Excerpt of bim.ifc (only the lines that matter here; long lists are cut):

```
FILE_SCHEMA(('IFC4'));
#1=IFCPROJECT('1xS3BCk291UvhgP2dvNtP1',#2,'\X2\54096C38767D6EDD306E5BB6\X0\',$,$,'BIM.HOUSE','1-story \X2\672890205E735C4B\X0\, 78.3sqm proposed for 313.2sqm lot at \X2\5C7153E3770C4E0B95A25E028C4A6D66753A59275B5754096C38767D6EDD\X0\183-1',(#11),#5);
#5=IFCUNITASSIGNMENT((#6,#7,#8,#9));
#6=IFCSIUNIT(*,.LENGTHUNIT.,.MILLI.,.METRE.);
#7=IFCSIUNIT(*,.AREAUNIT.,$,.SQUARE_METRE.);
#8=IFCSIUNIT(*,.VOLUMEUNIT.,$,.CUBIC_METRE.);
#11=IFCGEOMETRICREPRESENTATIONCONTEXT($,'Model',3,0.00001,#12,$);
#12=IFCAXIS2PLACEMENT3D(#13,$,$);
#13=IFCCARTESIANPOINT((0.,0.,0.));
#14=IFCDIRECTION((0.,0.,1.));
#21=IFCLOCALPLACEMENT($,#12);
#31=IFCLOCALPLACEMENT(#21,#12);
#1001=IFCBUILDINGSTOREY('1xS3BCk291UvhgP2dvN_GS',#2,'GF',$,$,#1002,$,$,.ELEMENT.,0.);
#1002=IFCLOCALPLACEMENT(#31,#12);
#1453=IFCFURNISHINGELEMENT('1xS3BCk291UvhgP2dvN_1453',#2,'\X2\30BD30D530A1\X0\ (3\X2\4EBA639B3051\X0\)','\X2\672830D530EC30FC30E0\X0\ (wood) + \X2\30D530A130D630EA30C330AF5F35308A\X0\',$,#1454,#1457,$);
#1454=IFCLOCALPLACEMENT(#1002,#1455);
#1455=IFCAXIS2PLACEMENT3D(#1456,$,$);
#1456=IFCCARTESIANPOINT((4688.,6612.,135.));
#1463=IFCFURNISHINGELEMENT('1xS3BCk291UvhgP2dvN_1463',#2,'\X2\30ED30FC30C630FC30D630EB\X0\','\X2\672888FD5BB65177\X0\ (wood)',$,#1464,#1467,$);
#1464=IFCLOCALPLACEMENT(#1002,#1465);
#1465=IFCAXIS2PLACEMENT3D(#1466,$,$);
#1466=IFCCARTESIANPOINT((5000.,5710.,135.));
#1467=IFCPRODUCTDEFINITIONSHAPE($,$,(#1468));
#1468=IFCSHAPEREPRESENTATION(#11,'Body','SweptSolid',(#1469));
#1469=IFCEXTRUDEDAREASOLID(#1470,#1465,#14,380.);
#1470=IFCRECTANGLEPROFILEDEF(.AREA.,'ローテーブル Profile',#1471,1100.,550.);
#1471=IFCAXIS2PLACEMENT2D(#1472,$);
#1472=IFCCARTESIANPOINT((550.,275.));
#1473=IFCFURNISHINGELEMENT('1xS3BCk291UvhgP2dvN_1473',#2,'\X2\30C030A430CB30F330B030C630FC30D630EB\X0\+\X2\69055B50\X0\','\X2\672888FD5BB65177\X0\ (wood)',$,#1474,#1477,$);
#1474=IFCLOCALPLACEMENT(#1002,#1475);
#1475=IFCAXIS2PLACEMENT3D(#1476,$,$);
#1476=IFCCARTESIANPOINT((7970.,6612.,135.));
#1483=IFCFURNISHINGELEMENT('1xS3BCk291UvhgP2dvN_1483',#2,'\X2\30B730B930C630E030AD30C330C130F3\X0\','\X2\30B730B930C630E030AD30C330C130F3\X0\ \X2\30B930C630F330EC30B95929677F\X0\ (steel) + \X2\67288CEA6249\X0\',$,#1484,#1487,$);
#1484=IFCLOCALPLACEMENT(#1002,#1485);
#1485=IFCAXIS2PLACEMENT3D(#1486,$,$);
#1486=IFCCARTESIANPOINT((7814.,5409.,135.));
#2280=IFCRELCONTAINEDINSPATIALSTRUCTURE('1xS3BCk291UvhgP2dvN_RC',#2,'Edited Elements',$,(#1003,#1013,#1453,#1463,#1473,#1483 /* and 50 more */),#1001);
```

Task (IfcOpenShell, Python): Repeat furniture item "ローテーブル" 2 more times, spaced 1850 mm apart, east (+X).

```python
import numpy as np
import ifcopenshell
import ifcopenshell.api.geometry
import ifcopenshell.api.root
import ifcopenshell.util.element
import ifcopenshell.util.placement
import ifcopenshell.util.unit

model = ifcopenshell.open("bim.ifc")
unit_scale = ifcopenshell.util.unit.calculate_unit_scale(model)


def reuse_history(source, copy):
    """copy_class also copies each property set's owner history, people and application; keep the originals."""
    for rel in copy.IsDefinedBy:
        if rel.is_a("IfcRelDefinesByProperties") and (history := rel.RelatingPropertyDefinition.OwnerHistory):
            rel.RelatingPropertyDefinition.OwnerHistory = source.OwnerHistory
            ifcopenshell.util.element.remove_deep2(model, history)


source = model.by_guid("1xS3BCk291UvhgP2dvN_1463")
base = ifcopenshell.util.placement.get_local_placement(source.ObjectPlacement)
step = np.array([1.0, 0.0, 0.0]) * 1.85 / unit_scale

for i in range(1, 3):
    copy = ifcopenshell.api.root.copy_class(model, product=source)
    copy.Representation = ifcopenshell.util.element.copy_deep(
        model, source.Representation, exclude=["IfcGeometricRepresentationContext", "IfcRepresentationMap"]
    )
    reuse_history(source, copy)
    matrix = base.copy()
    matrix[:3, 3] += i * step
    print("added at", matrix[:3, 3].round(3) + 0.0)
    ifcopenshell.api.geometry.edit_object_placement(model, product=copy, matrix=matrix, is_si=False)

model.write("bim_v2.ifc")
```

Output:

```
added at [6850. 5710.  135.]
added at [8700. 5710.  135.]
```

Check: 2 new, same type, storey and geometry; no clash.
